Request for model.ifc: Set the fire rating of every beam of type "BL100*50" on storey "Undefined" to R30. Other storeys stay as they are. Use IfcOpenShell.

First a look at what the model holds.

```python
import ifcopenshell
import ifcopenshell.util.element

model = ifcopenshell.open("model.ifc")
print(model.schema)
storey = next(s for s in model.by_type("IfcBuildingStorey") if s.Name == "Undefined")
beams = [e for e in ifcopenshell.util.element.get_decomposition(storey) if e.is_a("IfcBeam")]
seen = {}
for e in beams:
    element_type = ifcopenshell.util.element.get_type(e)
    key = (element_type.Name if element_type != e and element_type else None, ifcopenshell.util.element.get_pset(e, "Pset_BeamCommon", "FireRating"))
    seen[key] = seen.get(key, 0) + 1
for (name, value), count in sorted(seen.items(), key=str):
    print(count, "x", name, "|", value)
```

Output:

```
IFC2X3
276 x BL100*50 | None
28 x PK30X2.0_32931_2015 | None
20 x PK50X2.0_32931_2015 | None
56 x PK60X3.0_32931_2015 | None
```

```python
import ifcopenshell
import ifcopenshell.api.pset
import ifcopenshell.util.element

model = ifcopenshell.open("model.ifc")

storey = next(s for s in model.by_type("IfcBuildingStorey") if s.Name == "Undefined")
beams = [e for e in ifcopenshell.util.element.get_decomposition(storey) if e.is_a("IfcBeam")]

count = 0
for e in beams:
    element_type = ifcopenshell.util.element.get_type(e)
    if element_type in (None, e) or element_type.Name != "BL100*50":
        continue
    found = ifcopenshell.util.element.get_pset(e, "Pset_BeamCommon", should_inherit=False)
    if found:
        pset = model.by_id(found["id"])
        if len(ifcopenshell.util.element.get_elements_by_pset(pset)) > 1:
            pset = ifcopenshell.api.pset.unshare_pset(model, products=[e], pset=pset)[0]
    else:
        pset = ifcopenshell.api.pset.add_pset(model, product=e, name="Pset_BeamCommon")
    ifcopenshell.api.pset.edit_pset(model, pset=pset, properties={"FireRating": "R30"})
    count += 1

print(count, "beams updated")

model.write("model_updated.ifc")
```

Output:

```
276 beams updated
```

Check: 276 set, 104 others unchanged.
